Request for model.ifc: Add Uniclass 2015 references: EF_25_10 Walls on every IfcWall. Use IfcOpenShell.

First a look at what the model holds.

```python
import ifcopenshell

model = ifcopenshell.open("model.ifc")
print(model.schema)
print("classifications:", [c.Name for c in model.by_type("IfcClassification")])
for ifc_class in ("IfcDoor", "IfcRoof", "IfcStair", "IfcWall", "IfcWindow"):
    print(ifc_class, len(model.by_type(ifc_class)))
```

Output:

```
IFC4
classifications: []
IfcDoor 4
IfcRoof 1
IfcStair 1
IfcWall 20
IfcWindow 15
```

```python
import ifcopenshell
import ifcopenshell.api.classification

model = ifcopenshell.open("model.ifc")

system = ifcopenshell.api.classification.add_classification(model, classification="Uniclass 2015")

codes = {
    "IfcWall": ("EF_25_10", "Walls"),
}
for ifc_class, (code, name) in codes.items():
    products = model.by_type(ifc_class)
    ifcopenshell.api.classification.add_reference(
        model, products=products, classification=system, identification=code, name=name
    )
    print(code, len(products))

model.write("model_v2.ifc")
```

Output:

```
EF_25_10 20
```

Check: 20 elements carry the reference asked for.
